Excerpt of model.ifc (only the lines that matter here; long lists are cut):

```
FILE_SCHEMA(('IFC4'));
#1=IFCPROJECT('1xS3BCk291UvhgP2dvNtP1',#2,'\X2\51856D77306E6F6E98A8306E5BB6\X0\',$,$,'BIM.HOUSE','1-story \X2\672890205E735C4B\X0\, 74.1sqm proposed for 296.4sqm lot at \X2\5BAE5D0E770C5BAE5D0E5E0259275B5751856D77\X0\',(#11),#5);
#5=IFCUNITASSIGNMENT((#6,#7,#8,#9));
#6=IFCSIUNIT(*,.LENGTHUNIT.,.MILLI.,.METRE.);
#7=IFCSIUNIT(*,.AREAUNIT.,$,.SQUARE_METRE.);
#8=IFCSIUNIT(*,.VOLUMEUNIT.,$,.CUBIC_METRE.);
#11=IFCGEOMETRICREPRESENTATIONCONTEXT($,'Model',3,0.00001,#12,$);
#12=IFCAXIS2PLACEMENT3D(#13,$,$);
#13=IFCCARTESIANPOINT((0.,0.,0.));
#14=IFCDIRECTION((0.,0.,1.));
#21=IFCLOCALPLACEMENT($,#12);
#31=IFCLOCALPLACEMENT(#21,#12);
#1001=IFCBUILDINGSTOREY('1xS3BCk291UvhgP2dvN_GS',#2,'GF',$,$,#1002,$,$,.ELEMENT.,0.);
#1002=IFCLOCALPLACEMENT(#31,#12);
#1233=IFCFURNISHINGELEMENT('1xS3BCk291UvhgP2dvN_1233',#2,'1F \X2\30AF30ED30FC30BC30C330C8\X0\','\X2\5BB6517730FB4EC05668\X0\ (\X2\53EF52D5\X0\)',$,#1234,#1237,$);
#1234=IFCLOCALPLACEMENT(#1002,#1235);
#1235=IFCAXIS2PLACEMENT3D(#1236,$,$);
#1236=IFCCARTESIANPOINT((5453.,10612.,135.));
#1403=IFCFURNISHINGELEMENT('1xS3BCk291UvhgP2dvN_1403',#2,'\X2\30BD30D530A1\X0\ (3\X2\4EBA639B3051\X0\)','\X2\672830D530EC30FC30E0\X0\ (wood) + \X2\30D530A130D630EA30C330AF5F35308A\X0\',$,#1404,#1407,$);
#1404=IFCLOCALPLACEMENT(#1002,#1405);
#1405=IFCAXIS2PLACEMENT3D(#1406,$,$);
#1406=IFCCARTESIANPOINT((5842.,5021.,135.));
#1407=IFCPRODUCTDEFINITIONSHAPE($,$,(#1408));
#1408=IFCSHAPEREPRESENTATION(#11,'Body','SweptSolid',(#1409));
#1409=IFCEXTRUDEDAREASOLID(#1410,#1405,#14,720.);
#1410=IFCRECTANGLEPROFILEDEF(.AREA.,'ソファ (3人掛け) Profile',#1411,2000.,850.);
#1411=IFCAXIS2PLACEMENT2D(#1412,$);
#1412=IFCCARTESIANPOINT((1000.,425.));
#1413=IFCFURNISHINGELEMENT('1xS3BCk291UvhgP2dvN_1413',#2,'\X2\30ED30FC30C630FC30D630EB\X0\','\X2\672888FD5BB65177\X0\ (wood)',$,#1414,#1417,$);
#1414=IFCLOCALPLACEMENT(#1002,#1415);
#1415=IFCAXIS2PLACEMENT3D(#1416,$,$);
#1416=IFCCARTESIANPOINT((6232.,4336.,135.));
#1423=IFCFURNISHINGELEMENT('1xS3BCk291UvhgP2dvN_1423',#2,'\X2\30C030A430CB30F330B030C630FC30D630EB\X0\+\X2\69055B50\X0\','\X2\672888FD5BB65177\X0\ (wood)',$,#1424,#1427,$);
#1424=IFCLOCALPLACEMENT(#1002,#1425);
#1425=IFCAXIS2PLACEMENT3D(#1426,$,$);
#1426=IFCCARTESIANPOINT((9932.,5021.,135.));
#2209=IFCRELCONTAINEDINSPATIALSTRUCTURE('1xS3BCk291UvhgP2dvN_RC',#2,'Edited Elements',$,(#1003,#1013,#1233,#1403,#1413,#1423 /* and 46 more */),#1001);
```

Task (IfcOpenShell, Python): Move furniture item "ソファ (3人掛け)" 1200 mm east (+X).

```python
import ifcopenshell
import ifcopenshell.api.geometry
import ifcopenshell.util.placement
import ifcopenshell.util.unit

model = ifcopenshell.open("model.ifc")
unit_scale = ifcopenshell.util.unit.calculate_unit_scale(model)

item = model.by_guid("1xS3BCk291UvhgP2dvN_1403")
matrix = ifcopenshell.util.placement.get_local_placement(item.ObjectPlacement)
matrix[0, 3] += 1.2 / unit_scale
ifcopenshell.api.geometry.edit_object_placement(model, product=item, matrix=matrix, is_si=False)

print(ifcopenshell.util.placement.get_local_placement(item.ObjectPlacement).round(3) + 0.0)

model.write("model_rev.ifc")
```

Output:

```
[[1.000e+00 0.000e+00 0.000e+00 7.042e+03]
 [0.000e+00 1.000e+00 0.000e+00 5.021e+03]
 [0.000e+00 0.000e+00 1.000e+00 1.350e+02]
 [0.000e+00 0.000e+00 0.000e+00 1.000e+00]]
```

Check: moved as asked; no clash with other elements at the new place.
